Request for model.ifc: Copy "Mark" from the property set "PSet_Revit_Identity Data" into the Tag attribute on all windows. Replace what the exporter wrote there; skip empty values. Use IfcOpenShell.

First a look at what the model holds.

```python
import ifcopenshell
import ifcopenshell.util.element

model = ifcopenshell.open("model.ifc")
print(model.schema)
windows = model.by_type("IfcWindow")
print(len(windows), "windows")
for e in windows[:8]:
    source = ifcopenshell.util.element.get_pset(e, "PSet_Revit_Identity Data", "Mark")
    target = e.Tag
    print(e.id(), repr(source), repr(target), sep=" | ")
```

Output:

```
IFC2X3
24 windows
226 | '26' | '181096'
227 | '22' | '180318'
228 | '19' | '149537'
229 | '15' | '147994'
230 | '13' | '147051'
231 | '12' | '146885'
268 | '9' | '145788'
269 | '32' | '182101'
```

```python
import ifcopenshell
import ifcopenshell.util.element

model = ifcopenshell.open("model.ifc")

count = 0
for e in model.by_type("IfcWindow"):
    value = ifcopenshell.util.element.get_pset(e, "PSet_Revit_Identity Data", "Mark")
    current = e.Tag
    if not value or not value.strip() or current == value:
        continue
    e.Tag = value
    count += 1

print(count, "windows updated")

model.write("model_rev.ifc")
```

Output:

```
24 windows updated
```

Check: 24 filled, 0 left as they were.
